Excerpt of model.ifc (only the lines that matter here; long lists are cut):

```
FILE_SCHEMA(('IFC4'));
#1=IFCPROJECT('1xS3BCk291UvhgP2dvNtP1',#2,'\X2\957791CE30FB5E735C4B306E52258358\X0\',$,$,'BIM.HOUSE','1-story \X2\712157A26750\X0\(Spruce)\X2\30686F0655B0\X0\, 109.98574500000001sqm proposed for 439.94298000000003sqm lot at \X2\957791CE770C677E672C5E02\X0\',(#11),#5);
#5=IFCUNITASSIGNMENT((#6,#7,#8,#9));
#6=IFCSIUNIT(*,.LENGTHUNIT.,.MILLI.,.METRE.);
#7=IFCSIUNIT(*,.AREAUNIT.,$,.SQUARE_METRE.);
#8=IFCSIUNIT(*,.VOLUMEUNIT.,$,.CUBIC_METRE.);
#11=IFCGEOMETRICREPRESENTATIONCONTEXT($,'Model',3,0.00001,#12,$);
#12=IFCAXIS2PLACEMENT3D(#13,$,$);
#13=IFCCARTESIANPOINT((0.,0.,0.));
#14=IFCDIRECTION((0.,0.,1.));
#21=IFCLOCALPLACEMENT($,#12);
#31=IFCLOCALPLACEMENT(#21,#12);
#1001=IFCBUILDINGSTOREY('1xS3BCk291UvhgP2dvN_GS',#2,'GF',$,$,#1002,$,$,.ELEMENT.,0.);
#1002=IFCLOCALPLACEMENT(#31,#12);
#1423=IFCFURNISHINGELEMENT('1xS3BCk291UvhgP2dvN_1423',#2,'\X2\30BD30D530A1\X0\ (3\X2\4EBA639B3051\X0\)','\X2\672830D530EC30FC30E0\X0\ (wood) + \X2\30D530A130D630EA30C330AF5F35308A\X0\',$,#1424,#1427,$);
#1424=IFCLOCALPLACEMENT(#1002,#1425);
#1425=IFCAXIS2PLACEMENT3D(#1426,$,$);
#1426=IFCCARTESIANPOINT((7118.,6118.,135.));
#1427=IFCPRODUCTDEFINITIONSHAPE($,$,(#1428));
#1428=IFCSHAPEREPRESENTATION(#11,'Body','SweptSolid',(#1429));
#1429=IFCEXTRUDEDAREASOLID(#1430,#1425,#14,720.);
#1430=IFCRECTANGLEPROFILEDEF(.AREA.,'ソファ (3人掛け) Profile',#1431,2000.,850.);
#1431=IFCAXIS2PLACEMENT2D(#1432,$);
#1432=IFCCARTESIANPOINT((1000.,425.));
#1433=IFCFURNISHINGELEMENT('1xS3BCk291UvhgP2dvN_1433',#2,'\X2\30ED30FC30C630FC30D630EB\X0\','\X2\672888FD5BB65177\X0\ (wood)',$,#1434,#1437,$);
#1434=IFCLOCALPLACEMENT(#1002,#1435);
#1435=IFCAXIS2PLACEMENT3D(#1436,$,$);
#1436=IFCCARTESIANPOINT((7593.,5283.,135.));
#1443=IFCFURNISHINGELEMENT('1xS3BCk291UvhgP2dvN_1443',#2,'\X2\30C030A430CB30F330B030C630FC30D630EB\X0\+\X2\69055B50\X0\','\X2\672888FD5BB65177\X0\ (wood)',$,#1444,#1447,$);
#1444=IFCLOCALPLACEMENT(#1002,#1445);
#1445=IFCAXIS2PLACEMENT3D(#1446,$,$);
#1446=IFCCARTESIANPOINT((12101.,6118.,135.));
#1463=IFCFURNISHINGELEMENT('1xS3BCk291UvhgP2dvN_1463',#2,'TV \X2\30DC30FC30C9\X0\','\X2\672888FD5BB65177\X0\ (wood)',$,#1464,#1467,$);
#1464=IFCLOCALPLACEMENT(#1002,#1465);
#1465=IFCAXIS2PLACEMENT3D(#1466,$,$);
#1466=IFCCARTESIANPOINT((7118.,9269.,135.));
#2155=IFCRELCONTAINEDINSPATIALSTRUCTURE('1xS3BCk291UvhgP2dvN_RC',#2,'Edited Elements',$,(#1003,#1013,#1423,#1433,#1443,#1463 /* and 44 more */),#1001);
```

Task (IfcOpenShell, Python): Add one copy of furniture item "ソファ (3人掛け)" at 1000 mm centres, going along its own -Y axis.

```python
import ifcopenshell
import ifcopenshell.api.geometry
import ifcopenshell.api.root
import ifcopenshell.util.element
import ifcopenshell.util.placement

model = ifcopenshell.open("model.ifc")


def reuse_history(source, copy):
    """copy_class also copies each property set's owner history, people and application; keep the originals."""
    for rel in copy.IsDefinedBy:
        if rel.is_a("IfcRelDefinesByProperties") and (history := rel.RelatingPropertyDefinition.OwnerHistory):
            rel.RelatingPropertyDefinition.OwnerHistory = source.OwnerHistory
            ifcopenshell.util.element.remove_deep2(model, history)


source = model.by_guid("1xS3BCk291UvhgP2dvN_1423")
base = ifcopenshell.util.placement.get_local_placement(source.ObjectPlacement)
step = -base[:3, 1] * 1000.0

for i in range(1, 2):
    copy = ifcopenshell.api.root.copy_class(model, product=source)
    copy.Representation = ifcopenshell.util.element.copy_deep(
        model, source.Representation, exclude=["IfcGeometricRepresentationContext", "IfcRepresentationMap"]
    )
    reuse_history(source, copy)
    matrix = base.copy()
    matrix[:3, 3] += i * step
    print("added at", matrix[:3, 3].round(3) + 0.0)
    ifcopenshell.api.geometry.edit_object_placement(model, product=copy, matrix=matrix, is_si=False)

model.write("model_rev.ifc")
```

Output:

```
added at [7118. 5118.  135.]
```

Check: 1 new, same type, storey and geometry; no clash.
